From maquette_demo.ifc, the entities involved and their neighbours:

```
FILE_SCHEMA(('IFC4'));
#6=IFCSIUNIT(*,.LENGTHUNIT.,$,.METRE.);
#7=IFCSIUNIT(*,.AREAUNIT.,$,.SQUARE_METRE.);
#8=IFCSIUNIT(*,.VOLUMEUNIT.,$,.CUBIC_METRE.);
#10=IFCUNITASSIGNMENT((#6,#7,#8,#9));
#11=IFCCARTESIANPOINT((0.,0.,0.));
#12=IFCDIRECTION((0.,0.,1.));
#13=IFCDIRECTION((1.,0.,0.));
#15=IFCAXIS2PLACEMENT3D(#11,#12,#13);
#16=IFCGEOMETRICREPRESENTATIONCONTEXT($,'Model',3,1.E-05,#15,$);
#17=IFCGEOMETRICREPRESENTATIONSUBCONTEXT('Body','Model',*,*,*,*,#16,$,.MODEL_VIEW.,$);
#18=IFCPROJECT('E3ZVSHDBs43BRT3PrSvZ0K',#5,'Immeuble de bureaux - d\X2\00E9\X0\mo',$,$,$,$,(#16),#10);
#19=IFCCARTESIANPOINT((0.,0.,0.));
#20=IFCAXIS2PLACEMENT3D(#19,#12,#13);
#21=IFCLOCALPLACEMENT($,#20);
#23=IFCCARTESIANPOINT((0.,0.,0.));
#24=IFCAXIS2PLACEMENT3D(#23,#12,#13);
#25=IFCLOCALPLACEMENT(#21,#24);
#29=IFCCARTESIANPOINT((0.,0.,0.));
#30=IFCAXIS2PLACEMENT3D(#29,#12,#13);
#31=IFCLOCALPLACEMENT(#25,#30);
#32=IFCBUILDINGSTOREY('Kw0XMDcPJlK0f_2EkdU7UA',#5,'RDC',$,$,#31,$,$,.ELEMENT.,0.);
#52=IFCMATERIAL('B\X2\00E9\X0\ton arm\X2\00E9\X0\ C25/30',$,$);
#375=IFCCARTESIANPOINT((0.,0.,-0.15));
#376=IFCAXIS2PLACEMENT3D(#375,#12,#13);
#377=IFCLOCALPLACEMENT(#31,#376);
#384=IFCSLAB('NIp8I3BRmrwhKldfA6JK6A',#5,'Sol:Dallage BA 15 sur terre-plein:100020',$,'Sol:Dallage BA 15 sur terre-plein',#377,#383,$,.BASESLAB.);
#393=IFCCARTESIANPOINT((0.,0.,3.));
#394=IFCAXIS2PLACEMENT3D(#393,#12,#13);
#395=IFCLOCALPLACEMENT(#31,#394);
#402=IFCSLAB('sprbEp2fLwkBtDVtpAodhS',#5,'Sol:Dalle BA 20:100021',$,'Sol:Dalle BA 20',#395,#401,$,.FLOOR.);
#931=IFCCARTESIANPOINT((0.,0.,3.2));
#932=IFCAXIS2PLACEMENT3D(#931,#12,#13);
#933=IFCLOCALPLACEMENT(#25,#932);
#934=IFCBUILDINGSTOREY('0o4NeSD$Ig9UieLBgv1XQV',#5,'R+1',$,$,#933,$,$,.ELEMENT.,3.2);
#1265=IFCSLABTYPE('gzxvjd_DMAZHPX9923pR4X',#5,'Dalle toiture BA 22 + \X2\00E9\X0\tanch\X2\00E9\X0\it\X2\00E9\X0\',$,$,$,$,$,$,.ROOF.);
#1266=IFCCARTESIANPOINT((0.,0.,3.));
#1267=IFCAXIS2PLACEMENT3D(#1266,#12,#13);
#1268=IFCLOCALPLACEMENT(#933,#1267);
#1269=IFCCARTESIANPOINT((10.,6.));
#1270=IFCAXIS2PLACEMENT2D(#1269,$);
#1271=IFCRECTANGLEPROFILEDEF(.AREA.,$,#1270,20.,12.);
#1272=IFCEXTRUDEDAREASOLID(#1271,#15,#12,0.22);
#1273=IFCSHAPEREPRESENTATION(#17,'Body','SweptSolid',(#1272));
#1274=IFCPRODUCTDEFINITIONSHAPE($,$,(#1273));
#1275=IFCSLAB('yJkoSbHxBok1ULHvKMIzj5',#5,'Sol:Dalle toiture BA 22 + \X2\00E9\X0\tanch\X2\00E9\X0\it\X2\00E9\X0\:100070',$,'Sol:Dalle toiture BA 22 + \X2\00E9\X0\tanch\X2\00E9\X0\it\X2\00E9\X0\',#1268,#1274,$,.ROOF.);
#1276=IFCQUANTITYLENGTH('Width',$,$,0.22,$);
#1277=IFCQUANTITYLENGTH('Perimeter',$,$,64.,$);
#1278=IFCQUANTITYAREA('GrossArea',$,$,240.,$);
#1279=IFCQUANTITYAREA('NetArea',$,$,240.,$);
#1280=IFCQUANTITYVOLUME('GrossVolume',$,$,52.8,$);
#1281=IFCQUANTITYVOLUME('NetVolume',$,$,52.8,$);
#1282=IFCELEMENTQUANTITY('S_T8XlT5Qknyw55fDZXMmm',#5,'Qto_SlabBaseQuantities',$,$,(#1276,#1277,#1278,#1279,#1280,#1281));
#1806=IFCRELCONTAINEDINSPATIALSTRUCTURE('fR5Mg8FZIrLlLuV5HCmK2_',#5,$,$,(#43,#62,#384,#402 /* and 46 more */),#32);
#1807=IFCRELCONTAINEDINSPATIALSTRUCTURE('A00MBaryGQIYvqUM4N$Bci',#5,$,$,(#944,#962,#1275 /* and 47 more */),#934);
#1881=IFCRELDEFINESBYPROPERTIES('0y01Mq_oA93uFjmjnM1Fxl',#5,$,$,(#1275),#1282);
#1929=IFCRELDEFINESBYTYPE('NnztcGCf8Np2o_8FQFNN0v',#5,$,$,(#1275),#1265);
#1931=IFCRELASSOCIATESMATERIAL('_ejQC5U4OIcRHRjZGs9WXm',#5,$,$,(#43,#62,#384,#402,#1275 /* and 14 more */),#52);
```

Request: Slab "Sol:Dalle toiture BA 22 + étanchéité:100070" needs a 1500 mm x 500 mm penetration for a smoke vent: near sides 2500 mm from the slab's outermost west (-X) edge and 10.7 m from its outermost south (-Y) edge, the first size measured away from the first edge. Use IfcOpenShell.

```python
import numpy as np
import ifcopenshell
import ifcopenshell.api.feature
import ifcopenshell.api.geometry
import ifcopenshell.api.pset
import ifcopenshell.api.root
import ifcopenshell.geom
import ifcopenshell.util.element
import ifcopenshell.util.placement
import ifcopenshell.util.representation
import ifcopenshell.util.shape
import ifcopenshell.util.unit

model = ifcopenshell.open("maquette_demo.ifc")
unit_scale = ifcopenshell.util.unit.calculate_unit_scale(model)
area_scale = ifcopenshell.util.unit.calculate_unit_scale(model, "AREAUNIT")
volume_scale = ifcopenshell.util.unit.calculate_unit_scale(model, "VOLUMEUNIT")
settings = ifcopenshell.geom.settings()


def volume(element):
    """Net volume in cubic metres, openings subtracted."""
    shape = ifcopenshell.geom.create_shape(settings, element)
    return ifcopenshell.util.shape.get_volume(shape.geometry)


slab = model.by_guid("yJkoSbHxBok1ULHvKMIzj5")
before = volume(slab)

# Extent in the slab's own axes, in metres. The edges named are its -X and -Y sides.
slab_shape = ifcopenshell.geom.create_shape(settings, slab)
vertices = ifcopenshell.util.shape.get_vertices(slab_shape.geometry)
x_min, y_min, bottom = vertices.min(axis=0)
top = vertices[:, 2].max()

opening = ifcopenshell.api.root.create_entity(model, ifc_class="IfcOpeningElement", name="Smoke vent opening", predefined_type="OPENING")
context = ifcopenshell.util.representation.get_context(model, "Model", "Body", "MODEL_VIEW")
width, depth = 1.5, 0.5
outline = [(0.0, 0.0), (width, 0.0), (width, depth), (0.0, depth), (0.0, 0.0)]
# Overshoot both faces by 50 mm so the cut is clean.
shape = ifcopenshell.api.geometry.add_slab_representation(
    model, context=context, depth=top - bottom + 0.1, polyline=outline
)
ifcopenshell.api.geometry.assign_representation(model, product=opening, representation=shape)

matrix = ifcopenshell.util.placement.get_local_placement(slab.ObjectPlacement)
matrix[:, 3] = matrix @ np.append(np.array([x_min + 2.5, y_min + 10.7, bottom - 0.05]) / unit_scale, 1.0)
ifcopenshell.api.geometry.edit_object_placement(model, product=opening, matrix=matrix, is_si=False)
ifcopenshell.api.feature.add_feature(model, feature=opening, element=slab)

after = volume(slab)

# Update the slab's stored quantities.
qto = model.by_id(ifcopenshell.util.element.get_pset(slab, "Qto_SlabBaseQuantities", should_inherit=False)["id"])
ifcopenshell.api.pset.edit_qto(model, qto=qto, properties={
    "NetArea": after / (top - bottom) / area_scale,
    "NetVolume": after / volume_scale,
})

print(f"slab volume {before:.3f} -> {after:.3f} m3")

model.write("maquette_demo_edited.ifc")
```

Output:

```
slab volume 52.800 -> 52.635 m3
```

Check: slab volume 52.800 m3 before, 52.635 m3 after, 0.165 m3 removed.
